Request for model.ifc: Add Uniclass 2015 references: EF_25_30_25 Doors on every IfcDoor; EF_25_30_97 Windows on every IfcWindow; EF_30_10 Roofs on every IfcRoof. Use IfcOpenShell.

First a look at what the model holds.

```python
import ifcopenshell

model = ifcopenshell.open("model.ifc")
print(model.schema)
print("classifications:", [c.Name for c in model.by_type("IfcClassification")])
for ifc_class in ("IfcDoor", "IfcRoof", "IfcStair", "IfcWall", "IfcWindow"):
    print(ifc_class, len(model.by_type(ifc_class)))
```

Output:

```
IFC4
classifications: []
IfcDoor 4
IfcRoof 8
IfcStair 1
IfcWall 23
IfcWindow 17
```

```python
import ifcopenshell
import ifcopenshell.api.classification

model = ifcopenshell.open("model.ifc")

system = ifcopenshell.api.classification.add_classification(model, classification="Uniclass 2015")

codes = {
    "IfcDoor": ("EF_25_30_25", "Doors"),
    "IfcWindow": ("EF_25_30_97", "Windows"),
    "IfcRoof": ("EF_30_10", "Roofs"),
}
for ifc_class, (code, name) in codes.items():
    products = model.by_type(ifc_class)
    ifcopenshell.api.classification.add_reference(
        model, products=products, classification=system, identification=code, name=name
    )
    print(code, len(products))

model.write("model-out.ifc")
```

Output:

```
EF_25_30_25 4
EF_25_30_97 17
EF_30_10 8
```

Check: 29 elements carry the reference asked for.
